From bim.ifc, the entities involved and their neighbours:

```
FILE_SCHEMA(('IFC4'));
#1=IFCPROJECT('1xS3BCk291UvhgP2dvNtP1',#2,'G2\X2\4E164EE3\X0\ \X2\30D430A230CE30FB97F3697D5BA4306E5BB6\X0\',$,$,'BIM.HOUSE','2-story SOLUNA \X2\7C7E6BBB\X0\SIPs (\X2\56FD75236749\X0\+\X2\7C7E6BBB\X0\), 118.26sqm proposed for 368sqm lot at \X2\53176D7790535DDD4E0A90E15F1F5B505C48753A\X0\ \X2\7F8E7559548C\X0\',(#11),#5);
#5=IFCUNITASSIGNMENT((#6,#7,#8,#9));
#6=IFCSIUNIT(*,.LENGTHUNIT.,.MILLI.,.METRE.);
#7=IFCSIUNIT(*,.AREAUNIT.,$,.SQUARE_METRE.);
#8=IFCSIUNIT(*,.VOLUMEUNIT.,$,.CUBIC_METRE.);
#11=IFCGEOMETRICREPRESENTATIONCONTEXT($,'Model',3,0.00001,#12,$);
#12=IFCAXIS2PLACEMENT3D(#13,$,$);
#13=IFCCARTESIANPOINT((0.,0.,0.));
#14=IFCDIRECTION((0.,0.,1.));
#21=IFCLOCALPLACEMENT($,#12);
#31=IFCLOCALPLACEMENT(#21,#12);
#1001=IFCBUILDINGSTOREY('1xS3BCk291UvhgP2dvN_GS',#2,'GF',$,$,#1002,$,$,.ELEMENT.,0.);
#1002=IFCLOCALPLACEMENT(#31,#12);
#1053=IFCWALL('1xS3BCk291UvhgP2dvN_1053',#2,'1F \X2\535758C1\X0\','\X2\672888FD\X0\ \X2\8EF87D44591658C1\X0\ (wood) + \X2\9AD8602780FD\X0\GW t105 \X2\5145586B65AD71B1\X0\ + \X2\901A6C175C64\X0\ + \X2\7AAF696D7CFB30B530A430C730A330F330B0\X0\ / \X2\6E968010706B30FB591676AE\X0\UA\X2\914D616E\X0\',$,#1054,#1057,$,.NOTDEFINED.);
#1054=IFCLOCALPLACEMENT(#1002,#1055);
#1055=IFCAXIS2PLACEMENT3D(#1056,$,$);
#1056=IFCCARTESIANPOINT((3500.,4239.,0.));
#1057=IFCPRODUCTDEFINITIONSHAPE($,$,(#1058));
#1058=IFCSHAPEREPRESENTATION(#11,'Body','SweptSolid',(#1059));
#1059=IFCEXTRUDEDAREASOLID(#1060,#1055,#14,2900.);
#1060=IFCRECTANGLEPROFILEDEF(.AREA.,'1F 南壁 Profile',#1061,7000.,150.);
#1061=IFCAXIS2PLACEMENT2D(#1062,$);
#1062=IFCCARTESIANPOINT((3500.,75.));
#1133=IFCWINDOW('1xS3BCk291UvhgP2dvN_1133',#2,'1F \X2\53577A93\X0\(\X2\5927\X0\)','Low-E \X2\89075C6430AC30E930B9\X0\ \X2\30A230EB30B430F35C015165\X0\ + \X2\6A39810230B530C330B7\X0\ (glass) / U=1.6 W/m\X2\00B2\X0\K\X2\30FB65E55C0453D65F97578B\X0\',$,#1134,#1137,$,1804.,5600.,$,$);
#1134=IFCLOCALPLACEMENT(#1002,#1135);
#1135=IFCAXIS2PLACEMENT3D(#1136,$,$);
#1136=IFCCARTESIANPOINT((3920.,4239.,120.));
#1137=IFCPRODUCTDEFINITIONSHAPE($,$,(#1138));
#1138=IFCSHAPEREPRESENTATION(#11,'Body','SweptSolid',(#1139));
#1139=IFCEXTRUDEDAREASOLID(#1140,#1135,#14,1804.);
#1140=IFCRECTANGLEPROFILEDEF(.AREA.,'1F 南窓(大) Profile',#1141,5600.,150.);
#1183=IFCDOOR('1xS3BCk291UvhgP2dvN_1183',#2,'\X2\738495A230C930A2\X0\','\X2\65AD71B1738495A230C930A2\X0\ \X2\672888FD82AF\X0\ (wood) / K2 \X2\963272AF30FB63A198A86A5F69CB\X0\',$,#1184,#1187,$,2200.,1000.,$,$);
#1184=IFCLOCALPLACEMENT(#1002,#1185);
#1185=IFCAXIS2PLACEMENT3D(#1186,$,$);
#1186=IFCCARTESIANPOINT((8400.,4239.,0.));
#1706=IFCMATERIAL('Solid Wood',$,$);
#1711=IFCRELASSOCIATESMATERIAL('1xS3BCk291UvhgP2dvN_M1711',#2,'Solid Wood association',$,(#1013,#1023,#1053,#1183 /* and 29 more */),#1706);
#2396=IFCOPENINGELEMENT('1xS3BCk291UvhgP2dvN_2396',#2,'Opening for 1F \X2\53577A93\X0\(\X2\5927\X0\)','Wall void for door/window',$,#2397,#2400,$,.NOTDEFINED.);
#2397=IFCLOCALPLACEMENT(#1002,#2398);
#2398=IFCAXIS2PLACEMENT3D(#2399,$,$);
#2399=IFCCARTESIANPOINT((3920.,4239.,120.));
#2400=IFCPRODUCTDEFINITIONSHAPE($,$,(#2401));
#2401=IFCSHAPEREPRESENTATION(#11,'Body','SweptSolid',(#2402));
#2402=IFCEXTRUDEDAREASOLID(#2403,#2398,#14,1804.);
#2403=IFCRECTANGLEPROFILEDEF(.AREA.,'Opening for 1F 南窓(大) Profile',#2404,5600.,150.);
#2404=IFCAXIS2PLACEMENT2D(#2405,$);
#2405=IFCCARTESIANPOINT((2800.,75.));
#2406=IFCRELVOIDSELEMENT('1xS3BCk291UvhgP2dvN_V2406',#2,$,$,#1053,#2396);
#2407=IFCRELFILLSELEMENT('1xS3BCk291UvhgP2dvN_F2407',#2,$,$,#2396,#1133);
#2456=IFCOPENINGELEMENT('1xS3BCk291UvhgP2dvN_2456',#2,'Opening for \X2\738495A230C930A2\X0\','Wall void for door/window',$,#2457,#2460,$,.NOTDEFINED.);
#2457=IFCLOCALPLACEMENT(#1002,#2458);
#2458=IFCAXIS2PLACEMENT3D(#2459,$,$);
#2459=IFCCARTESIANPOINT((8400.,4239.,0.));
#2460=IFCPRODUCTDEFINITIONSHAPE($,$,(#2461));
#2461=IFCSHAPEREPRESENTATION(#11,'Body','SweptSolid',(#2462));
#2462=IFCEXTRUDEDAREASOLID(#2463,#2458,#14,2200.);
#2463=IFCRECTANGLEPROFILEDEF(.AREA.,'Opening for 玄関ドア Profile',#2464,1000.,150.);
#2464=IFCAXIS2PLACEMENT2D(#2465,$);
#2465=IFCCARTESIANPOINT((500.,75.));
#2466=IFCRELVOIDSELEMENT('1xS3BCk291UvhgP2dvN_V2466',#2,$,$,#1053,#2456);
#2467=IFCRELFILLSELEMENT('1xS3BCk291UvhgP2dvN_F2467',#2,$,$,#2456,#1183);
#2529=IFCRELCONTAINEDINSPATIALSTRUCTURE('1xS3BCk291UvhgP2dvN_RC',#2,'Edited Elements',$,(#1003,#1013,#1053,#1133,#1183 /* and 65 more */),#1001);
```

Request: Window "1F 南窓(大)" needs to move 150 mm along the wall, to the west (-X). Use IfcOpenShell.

```python
import ifcopenshell
import ifcopenshell.api.geometry
import ifcopenshell.util.placement

model = ifcopenshell.open("bim.ifc")

window = model.by_guid("1xS3BCk291UvhgP2dvN_1133")
opening = window.FillsVoids[0].RelatingOpeningElement
wall = opening.VoidsElements[0].RelatingBuildingElement

wall_matrix = ifcopenshell.util.placement.get_local_placement(wall.ObjectPlacement)
shift = wall_matrix[:3, 0] * -150.0
before = ifcopenshell.util.placement.get_local_placement(window.ObjectPlacement)[:3, 3].copy()

# The window is not placed relative to its opening, so move both.
for product in (opening, window):
    matrix = ifcopenshell.util.placement.get_local_placement(product.ObjectPlacement)
    matrix[:3, 3] += shift
    ifcopenshell.api.geometry.edit_object_placement(model, product=product, matrix=matrix, is_si=False)

after = ifcopenshell.util.placement.get_local_placement(window.ObjectPlacement)[:3, 3]
print("window moved by", (after - before).round(3) + 0.0)

model.write("bim_updated.ifc")
```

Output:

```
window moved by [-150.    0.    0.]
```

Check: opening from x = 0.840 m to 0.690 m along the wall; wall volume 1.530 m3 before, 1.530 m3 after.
